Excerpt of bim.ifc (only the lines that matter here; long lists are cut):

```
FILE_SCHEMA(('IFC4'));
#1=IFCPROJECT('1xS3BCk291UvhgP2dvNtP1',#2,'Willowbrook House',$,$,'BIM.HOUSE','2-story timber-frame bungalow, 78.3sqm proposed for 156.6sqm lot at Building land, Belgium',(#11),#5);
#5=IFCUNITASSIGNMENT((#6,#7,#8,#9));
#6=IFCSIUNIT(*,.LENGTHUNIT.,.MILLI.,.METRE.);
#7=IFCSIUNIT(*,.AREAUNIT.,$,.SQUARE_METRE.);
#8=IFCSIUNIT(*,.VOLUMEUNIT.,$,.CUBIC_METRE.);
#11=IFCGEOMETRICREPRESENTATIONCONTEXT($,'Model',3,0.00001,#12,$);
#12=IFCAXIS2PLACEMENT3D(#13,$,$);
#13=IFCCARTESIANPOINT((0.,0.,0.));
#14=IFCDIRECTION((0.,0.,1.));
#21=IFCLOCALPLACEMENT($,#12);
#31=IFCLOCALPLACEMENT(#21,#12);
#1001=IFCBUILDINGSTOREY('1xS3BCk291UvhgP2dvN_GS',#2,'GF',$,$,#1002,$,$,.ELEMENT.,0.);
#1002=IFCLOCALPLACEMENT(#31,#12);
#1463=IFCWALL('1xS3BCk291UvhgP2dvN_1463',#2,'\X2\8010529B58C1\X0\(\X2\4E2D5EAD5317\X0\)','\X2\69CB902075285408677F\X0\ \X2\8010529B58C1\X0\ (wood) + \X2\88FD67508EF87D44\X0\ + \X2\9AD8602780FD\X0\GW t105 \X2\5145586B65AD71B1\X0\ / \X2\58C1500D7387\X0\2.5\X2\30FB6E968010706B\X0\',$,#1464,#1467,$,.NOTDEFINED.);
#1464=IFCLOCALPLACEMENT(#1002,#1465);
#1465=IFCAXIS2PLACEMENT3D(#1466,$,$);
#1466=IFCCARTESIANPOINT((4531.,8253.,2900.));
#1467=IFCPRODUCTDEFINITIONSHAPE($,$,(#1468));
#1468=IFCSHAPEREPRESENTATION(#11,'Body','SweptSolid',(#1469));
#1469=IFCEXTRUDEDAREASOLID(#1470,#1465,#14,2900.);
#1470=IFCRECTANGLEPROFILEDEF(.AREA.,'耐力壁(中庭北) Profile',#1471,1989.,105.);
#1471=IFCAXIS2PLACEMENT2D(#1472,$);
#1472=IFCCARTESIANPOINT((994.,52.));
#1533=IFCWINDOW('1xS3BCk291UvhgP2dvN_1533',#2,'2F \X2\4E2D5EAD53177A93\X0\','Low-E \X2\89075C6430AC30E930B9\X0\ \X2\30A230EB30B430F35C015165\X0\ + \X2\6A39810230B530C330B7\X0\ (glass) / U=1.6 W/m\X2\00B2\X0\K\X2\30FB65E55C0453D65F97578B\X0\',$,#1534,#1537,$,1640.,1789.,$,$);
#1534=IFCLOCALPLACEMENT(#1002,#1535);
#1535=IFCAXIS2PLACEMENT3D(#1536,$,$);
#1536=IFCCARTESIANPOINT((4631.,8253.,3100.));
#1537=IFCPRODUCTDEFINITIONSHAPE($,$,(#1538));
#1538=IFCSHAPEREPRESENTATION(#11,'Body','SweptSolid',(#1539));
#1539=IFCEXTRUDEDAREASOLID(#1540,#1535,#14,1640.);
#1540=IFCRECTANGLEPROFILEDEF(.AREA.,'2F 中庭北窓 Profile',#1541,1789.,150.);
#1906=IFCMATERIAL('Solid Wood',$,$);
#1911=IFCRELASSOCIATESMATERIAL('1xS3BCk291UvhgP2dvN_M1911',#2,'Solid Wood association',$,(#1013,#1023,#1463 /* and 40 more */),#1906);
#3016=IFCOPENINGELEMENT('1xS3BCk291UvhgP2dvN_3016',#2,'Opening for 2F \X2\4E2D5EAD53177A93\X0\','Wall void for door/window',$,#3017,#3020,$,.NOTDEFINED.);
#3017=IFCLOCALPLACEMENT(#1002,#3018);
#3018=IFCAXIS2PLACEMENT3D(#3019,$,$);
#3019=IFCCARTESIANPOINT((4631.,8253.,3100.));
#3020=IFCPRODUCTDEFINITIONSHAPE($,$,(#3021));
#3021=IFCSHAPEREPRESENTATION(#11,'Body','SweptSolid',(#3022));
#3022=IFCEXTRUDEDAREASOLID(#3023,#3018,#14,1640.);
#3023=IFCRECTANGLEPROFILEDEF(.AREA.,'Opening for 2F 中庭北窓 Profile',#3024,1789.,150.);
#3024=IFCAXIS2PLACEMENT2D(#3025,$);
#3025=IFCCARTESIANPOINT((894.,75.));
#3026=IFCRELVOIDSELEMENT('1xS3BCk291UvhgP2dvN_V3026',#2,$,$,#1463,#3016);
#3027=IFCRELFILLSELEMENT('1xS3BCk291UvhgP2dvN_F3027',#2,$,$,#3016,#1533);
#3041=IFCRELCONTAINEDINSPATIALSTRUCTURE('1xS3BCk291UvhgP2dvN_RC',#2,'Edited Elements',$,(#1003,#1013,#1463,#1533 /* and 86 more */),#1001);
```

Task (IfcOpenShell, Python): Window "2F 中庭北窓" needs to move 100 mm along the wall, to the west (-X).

```python
import ifcopenshell
import ifcopenshell.api.geometry
import ifcopenshell.util.placement
import ifcopenshell.util.unit

model = ifcopenshell.open("bim.ifc")
unit_scale = ifcopenshell.util.unit.calculate_unit_scale(model)

window = model.by_id(1533)
opening = window.FillsVoids[0].RelatingOpeningElement
wall = opening.VoidsElements[0].RelatingBuildingElement

wall_matrix = ifcopenshell.util.placement.get_local_placement(wall.ObjectPlacement)
shift = wall_matrix[:3, 0] * -0.1 / unit_scale
before = ifcopenshell.util.placement.get_local_placement(window.ObjectPlacement)[:3, 3].copy()

# The window is not placed relative to its opening, so move both.
for product in (opening, window):
    matrix = ifcopenshell.util.placement.get_local_placement(product.ObjectPlacement)
    matrix[:3, 3] += shift
    ifcopenshell.api.geometry.edit_object_placement(model, product=product, matrix=matrix, is_si=False)

after = ifcopenshell.util.placement.get_local_placement(window.ObjectPlacement)[:3, 3]
print("window moved by", (after - before).round(3) + 0.0)

model.write("bim_rev.ifc")
```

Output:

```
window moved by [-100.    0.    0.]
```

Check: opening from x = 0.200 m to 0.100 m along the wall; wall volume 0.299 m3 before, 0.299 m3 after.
